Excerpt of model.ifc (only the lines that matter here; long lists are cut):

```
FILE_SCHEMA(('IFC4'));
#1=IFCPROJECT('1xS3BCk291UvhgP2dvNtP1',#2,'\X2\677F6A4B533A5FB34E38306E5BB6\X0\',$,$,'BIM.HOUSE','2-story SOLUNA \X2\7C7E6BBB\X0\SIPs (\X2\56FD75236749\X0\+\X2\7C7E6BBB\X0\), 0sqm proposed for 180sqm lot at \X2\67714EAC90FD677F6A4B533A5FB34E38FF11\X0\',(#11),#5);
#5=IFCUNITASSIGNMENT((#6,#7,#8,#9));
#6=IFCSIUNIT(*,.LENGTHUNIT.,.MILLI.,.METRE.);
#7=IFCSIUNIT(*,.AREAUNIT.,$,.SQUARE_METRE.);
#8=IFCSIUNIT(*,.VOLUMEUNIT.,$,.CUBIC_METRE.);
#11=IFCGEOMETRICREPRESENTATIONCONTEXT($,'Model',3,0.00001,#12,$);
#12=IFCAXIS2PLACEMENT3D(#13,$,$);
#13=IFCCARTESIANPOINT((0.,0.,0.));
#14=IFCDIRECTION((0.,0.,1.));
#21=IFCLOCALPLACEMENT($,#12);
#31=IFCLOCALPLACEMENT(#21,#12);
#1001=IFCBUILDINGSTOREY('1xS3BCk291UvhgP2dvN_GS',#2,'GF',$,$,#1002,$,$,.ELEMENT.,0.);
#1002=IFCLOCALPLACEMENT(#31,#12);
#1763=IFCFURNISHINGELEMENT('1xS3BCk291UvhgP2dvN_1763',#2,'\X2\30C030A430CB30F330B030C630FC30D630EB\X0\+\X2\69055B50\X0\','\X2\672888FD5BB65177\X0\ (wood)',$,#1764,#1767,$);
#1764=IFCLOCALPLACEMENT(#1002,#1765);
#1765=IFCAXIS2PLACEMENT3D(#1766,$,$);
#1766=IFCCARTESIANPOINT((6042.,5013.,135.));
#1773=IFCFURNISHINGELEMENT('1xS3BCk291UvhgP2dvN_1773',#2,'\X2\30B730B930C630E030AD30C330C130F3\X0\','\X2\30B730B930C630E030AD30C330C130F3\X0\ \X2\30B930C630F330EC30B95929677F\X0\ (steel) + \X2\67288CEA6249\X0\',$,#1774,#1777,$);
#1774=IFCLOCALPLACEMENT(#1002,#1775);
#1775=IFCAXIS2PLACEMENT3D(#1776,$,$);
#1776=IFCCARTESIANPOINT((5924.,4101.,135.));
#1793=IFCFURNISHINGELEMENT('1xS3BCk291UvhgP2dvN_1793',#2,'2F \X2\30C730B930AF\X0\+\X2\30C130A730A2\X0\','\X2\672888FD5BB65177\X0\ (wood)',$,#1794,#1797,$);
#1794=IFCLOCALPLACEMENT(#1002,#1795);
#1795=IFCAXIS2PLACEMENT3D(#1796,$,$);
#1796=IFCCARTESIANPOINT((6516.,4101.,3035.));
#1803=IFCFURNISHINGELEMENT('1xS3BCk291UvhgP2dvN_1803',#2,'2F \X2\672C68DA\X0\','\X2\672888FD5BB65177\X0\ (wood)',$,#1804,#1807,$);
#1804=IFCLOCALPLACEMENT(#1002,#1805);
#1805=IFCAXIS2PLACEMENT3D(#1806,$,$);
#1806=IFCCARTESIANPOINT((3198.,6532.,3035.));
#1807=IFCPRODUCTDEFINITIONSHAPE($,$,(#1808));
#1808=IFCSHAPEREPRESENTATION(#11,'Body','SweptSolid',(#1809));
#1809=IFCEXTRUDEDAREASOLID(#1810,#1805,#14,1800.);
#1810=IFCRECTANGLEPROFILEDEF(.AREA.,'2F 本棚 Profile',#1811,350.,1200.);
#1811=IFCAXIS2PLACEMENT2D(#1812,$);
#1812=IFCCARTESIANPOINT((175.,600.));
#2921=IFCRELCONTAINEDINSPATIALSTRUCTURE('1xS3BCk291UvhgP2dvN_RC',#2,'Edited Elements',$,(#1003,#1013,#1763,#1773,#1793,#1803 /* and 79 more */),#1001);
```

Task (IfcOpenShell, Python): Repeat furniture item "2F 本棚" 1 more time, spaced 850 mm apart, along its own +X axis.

```python
import ifcopenshell
import ifcopenshell.api.geometry
import ifcopenshell.api.root
import ifcopenshell.util.element
import ifcopenshell.util.placement

model = ifcopenshell.open("model.ifc")


def reuse_history(source, copy):
    """copy_class also copies each property set's owner history, people and application; keep the originals."""
    for rel in copy.IsDefinedBy:
        if rel.is_a("IfcRelDefinesByProperties") and (history := rel.RelatingPropertyDefinition.OwnerHistory):
            rel.RelatingPropertyDefinition.OwnerHistory = source.OwnerHistory
            ifcopenshell.util.element.remove_deep2(model, history)


source = model.by_guid("1xS3BCk291UvhgP2dvN_1803")
base = ifcopenshell.util.placement.get_local_placement(source.ObjectPlacement)
step = base[:3, 0] * 850.0

for i in range(1, 2):
    copy = ifcopenshell.api.root.copy_class(model, product=source)
    copy.Representation = ifcopenshell.util.element.copy_deep(
        model, source.Representation, exclude=["IfcGeometricRepresentationContext", "IfcRepresentationMap"]
    )
    reuse_history(source, copy)
    matrix = base.copy()
    matrix[:3, 3] += i * step
    print("added at", matrix[:3, 3].round(3) + 0.0)
    ifcopenshell.api.geometry.edit_object_placement(model, product=copy, matrix=matrix, is_si=False)

model.write("model-out.ifc")
```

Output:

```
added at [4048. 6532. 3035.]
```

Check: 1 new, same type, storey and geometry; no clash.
